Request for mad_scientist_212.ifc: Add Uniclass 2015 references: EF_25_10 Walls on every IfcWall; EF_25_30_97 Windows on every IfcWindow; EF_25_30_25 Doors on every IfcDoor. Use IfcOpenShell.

First a look at what the model holds.

```python
import ifcopenshell

model = ifcopenshell.open("mad_scientist_212.ifc")
print(model.schema)
print("classifications:", [c.Name for c in model.by_type("IfcClassification")])
for ifc_class in ("IfcDoor", "IfcRoof", "IfcStair", "IfcWall", "IfcWindow"):
    print(ifc_class, len(model.by_type(ifc_class)))
```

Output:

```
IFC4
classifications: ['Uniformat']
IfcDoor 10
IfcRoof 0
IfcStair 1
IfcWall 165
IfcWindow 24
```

```python
import ifcopenshell
import ifcopenshell.api.classification

model = ifcopenshell.open("mad_scientist_212.ifc")

system = ifcopenshell.api.classification.add_classification(model, classification="Uniclass 2015")

codes = {
    "IfcWall": ("EF_25_10", "Walls"),
    "IfcWindow": ("EF_25_30_97", "Windows"),
    "IfcDoor": ("EF_25_30_25", "Doors"),
}
for ifc_class, (code, name) in codes.items():
    products = model.by_type(ifc_class)
    ifcopenshell.api.classification.add_reference(
        model, products=products, classification=system, identification=code, name=name
    )
    print(code, len(products))

model.write("mad_scientist_212_edited.ifc")
```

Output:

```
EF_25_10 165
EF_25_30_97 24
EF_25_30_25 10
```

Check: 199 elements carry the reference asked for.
